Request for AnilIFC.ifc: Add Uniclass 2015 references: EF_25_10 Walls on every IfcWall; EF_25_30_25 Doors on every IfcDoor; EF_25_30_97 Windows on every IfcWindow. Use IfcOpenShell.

First a look at what the model holds.

```python
import ifcopenshell

model = ifcopenshell.open("AnilIFC.ifc")
print(model.schema)
print("classifications:", [c.Name for c in model.by_type("IfcClassification")])
for ifc_class in ("IfcDoor", "IfcRoof", "IfcStair", "IfcWall", "IfcWindow"):
    print(ifc_class, len(model.by_type(ifc_class)))
```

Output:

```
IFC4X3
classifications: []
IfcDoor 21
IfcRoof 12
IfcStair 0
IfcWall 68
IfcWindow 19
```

```python
import ifcopenshell
import ifcopenshell.api.classification

model = ifcopenshell.open("AnilIFC.ifc")

system = ifcopenshell.api.classification.add_classification(model, classification="Uniclass 2015")

codes = {
    "IfcWall": ("EF_25_10", "Walls"),
    "IfcDoor": ("EF_25_30_25", "Doors"),
    "IfcWindow": ("EF_25_30_97", "Windows"),
}
for ifc_class, (code, name) in codes.items():
    products = model.by_type(ifc_class)
    ifcopenshell.api.classification.add_reference(
        model, products=products, classification=system, identification=code, name=name
    )
    print(code, len(products))

model.write("AnilIFC_v2.ifc")
```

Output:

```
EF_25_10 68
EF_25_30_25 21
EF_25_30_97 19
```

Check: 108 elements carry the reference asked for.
